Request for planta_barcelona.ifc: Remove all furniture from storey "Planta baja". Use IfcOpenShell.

First a look at what the model holds.

```python
import ifcopenshell
import ifcopenshell.util.element

model = ifcopenshell.open("planta_barcelona.ifc")
print(model.schema)
storey = next(s for s in model.by_type("IfcBuildingStorey") if s.Name == "Planta baja")
furniture = [e for e in ifcopenshell.util.element.get_decomposition(storey) if e.is_a("IfcFurnishingElement")]
seen = {}
for e in furniture:
    element_type = ifcopenshell.util.element.get_type(e)
    name = element_type.Name if element_type not in (None, e) else None
    seen[name] = seen.get(name, 0) + 1
for name, count in sorted(seen.items(), key=str):
    print(count, "x", name)
```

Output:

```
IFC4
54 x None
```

```python
import ifcopenshell
import ifcopenshell.api.root
import ifcopenshell.util.element

model = ifcopenshell.open("planta_barcelona.ifc")

storey = next(s for s in model.by_type("IfcBuildingStorey") if s.Name == "Planta baja")
furniture = [e for e in ifcopenshell.util.element.get_decomposition(storey) if e.is_a("IfcFurnishingElement")]

for e in furniture:
    ifcopenshell.api.root.remove_product(model, product=e)
print(len(furniture), "removed")

model.write("planta_barcelona-out.ifc")
```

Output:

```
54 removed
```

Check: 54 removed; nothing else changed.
